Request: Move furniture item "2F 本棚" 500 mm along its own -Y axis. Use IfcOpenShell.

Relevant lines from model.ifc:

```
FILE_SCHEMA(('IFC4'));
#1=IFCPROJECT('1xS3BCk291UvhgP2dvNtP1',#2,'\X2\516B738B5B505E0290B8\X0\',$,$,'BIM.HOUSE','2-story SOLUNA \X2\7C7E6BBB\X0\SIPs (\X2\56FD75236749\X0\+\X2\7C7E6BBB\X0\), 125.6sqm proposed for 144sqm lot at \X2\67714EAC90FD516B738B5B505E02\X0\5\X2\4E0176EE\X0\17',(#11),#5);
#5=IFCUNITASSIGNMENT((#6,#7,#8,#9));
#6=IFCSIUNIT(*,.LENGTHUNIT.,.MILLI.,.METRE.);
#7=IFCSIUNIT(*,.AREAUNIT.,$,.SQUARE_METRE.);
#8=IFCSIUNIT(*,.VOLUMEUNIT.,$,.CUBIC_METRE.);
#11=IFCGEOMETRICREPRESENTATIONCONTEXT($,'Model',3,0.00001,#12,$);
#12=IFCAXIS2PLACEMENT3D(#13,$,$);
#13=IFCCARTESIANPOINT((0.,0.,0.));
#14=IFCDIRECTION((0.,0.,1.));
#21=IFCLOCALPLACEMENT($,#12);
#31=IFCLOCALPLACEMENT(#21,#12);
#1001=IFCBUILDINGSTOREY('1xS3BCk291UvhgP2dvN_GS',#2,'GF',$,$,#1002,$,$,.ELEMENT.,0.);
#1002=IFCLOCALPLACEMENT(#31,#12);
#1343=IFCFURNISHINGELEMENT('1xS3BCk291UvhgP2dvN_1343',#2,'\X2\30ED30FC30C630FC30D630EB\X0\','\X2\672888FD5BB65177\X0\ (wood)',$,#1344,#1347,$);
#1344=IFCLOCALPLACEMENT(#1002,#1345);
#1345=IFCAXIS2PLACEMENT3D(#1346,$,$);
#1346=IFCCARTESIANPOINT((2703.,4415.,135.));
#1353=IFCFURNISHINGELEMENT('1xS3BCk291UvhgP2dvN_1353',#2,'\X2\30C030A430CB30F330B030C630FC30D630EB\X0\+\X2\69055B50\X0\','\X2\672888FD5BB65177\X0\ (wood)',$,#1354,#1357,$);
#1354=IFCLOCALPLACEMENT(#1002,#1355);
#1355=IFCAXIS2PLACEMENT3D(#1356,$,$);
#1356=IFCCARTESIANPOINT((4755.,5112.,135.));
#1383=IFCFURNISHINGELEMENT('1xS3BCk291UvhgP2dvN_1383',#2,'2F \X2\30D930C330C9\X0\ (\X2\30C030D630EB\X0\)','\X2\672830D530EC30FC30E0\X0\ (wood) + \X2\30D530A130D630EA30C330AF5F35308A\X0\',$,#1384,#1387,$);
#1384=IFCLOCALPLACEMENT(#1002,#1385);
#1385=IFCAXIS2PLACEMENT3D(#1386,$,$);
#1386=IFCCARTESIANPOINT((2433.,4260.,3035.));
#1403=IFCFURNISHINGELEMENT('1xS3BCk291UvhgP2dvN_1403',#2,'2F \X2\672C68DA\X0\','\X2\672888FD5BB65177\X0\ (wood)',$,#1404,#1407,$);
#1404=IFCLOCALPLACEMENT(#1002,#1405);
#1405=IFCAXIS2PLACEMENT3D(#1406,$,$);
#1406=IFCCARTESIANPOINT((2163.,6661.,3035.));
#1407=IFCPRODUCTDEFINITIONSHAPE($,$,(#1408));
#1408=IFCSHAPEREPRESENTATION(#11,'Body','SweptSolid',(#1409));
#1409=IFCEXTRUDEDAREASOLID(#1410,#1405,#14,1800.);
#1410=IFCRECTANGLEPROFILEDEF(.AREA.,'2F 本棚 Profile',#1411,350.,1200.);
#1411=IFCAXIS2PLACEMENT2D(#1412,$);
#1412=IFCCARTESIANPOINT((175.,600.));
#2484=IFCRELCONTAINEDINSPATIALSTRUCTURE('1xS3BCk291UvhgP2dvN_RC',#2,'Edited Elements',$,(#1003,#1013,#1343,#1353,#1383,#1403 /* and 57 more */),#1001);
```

```python
import ifcopenshell
import ifcopenshell.api.geometry
import ifcopenshell.util.placement
import ifcopenshell.util.unit

model = ifcopenshell.open("model.ifc")
unit_scale = ifcopenshell.util.unit.calculate_unit_scale(model)

item = model.by_id(1403)
matrix = ifcopenshell.util.placement.get_local_placement(item.ObjectPlacement)
matrix[:3, 3] -= matrix[:3, 1] * 0.5 / unit_scale
ifcopenshell.api.geometry.edit_object_placement(model, product=item, matrix=matrix, is_si=False)

print(ifcopenshell.util.placement.get_local_placement(item.ObjectPlacement).round(3) + 0.0)

model.write("model_updated.ifc")
```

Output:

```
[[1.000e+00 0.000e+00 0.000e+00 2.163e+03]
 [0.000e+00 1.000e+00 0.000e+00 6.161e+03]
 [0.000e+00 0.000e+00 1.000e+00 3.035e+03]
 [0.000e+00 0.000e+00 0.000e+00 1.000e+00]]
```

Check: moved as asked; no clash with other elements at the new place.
